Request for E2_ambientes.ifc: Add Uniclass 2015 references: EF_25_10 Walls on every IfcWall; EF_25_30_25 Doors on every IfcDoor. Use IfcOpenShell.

First a look at what the model holds.

```python
import ifcopenshell

model = ifcopenshell.open("E2_ambientes.ifc")
print(model.schema)
print("classifications:", [c.Name for c in model.by_type("IfcClassification")])
for ifc_class in ("IfcDoor", "IfcRoof", "IfcStair", "IfcWall", "IfcWindow"):
    print(ifc_class, len(model.by_type(ifc_class)))
```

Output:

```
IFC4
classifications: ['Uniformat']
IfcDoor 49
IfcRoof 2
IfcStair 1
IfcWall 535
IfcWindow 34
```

```python
import ifcopenshell
import ifcopenshell.api.classification

model = ifcopenshell.open("E2_ambientes.ifc")

system = ifcopenshell.api.classification.add_classification(model, classification="Uniclass 2015")

codes = {
    "IfcWall": ("EF_25_10", "Walls"),
    "IfcDoor": ("EF_25_30_25", "Doors"),
}
for ifc_class, (code, name) in codes.items():
    products = model.by_type(ifc_class)
    ifcopenshell.api.classification.add_reference(
        model, products=products, classification=system, identification=code, name=name
    )
    print(code, len(products))

model.write("E2_ambientes_rev.ifc")
```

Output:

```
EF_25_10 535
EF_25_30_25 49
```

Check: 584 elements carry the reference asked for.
